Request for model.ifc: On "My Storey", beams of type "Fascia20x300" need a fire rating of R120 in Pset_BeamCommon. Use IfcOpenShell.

First a look at what the model holds.

```python
import ifcopenshell
import ifcopenshell.util.element

model = ifcopenshell.open("model.ifc")
print(model.schema)
storey = next(s for s in model.by_type("IfcBuildingStorey") if s.Name == "My Storey")
beams = [e for e in ifcopenshell.util.element.get_decomposition(storey) if e.is_a("IfcBeam")]
seen = {}
for e in beams:
    element_type = ifcopenshell.util.element.get_type(e)
    key = (element_type.Name if element_type != e and element_type else None, ifcopenshell.util.element.get_pset(e, "Pset_BeamCommon", "FireRating"))
    seen[key] = seen.get(key, 0) + 1
for (name, value), count in sorted(seen.items(), key=str):
    print(count, "x", name, "|", value)
```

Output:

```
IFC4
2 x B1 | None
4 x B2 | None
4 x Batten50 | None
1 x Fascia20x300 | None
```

```python
import ifcopenshell
import ifcopenshell.api.pset
import ifcopenshell.util.element

model = ifcopenshell.open("model.ifc")

storey = next(s for s in model.by_type("IfcBuildingStorey") if s.Name == "My Storey")
beams = [e for e in ifcopenshell.util.element.get_decomposition(storey) if e.is_a("IfcBeam")]

count = 0
for e in beams:
    element_type = ifcopenshell.util.element.get_type(e)
    if element_type in (None, e) or element_type.Name != "Fascia20x300":
        continue
    # add_pset returns the element's existing set when there is one.
    pset = ifcopenshell.api.pset.add_pset(model, product=e, name="Pset_BeamCommon")
    ifcopenshell.api.pset.edit_pset(model, pset=pset, properties={"FireRating": "R120"})
    count += 1

print(count, "beams updated")

model.write("model_v2.ifc")
```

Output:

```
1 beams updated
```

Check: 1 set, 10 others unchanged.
